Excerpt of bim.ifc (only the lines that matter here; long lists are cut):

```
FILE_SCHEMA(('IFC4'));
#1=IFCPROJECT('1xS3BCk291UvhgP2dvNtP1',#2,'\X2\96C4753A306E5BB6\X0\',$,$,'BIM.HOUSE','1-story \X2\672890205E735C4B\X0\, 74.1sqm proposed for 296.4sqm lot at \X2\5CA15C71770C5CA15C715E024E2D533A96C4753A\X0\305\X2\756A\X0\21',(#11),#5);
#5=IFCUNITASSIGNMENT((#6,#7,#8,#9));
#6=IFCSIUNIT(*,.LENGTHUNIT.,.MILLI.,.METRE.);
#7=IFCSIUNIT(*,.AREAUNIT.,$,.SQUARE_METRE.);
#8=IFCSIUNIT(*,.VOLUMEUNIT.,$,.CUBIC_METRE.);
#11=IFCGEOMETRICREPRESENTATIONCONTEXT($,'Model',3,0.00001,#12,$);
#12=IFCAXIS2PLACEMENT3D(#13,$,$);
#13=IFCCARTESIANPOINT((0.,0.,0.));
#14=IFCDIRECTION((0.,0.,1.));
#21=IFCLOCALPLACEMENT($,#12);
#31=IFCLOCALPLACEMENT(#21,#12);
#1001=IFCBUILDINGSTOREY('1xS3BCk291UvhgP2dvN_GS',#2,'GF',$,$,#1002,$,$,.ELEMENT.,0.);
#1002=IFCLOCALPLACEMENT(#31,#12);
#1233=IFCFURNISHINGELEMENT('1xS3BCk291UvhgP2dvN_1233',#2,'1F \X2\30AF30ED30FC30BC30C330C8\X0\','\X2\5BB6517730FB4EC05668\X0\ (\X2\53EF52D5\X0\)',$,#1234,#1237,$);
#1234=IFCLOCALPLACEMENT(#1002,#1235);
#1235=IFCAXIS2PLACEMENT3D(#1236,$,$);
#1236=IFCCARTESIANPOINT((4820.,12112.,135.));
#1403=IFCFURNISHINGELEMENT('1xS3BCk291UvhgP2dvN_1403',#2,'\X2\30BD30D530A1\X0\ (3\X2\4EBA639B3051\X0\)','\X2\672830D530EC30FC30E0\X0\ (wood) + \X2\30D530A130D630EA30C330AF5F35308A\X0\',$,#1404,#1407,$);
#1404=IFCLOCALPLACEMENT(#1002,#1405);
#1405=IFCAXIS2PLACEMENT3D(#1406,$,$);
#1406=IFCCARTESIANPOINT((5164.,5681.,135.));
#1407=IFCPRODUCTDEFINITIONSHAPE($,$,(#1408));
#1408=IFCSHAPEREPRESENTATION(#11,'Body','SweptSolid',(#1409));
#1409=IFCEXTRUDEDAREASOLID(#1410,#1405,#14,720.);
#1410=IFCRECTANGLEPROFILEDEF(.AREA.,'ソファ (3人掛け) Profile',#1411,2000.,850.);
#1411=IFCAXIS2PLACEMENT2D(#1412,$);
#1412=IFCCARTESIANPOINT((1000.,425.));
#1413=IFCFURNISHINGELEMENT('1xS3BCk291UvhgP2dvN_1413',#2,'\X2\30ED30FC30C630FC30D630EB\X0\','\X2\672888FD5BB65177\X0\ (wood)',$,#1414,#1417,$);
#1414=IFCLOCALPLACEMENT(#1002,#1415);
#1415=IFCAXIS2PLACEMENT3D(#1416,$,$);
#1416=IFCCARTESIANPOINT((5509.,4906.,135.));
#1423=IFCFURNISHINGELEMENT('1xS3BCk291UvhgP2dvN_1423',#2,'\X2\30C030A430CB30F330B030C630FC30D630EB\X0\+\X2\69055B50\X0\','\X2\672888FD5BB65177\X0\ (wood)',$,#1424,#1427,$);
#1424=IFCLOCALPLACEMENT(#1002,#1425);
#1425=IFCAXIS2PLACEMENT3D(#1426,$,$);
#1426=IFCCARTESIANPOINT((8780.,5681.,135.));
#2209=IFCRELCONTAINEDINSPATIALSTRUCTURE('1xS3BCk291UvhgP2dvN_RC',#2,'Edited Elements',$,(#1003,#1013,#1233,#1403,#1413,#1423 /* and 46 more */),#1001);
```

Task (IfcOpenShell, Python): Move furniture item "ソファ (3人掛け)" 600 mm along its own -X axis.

```python
import ifcopenshell
import ifcopenshell.api.geometry
import ifcopenshell.util.placement
import ifcopenshell.util.unit

model = ifcopenshell.open("bim.ifc")
unit_scale = ifcopenshell.util.unit.calculate_unit_scale(model)

item = model.by_guid("1xS3BCk291UvhgP2dvN_1403")
matrix = ifcopenshell.util.placement.get_local_placement(item.ObjectPlacement)
matrix[:3, 3] -= matrix[:3, 0] * 0.6 / unit_scale
ifcopenshell.api.geometry.edit_object_placement(model, product=item, matrix=matrix, is_si=False)

print(ifcopenshell.util.placement.get_local_placement(item.ObjectPlacement).round(3) + 0.0)

model.write("bim_edited.ifc")
```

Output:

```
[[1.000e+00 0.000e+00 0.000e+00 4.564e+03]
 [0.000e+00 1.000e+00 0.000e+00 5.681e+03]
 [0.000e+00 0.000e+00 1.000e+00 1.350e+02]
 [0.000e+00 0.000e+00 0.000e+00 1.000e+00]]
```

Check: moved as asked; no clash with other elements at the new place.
